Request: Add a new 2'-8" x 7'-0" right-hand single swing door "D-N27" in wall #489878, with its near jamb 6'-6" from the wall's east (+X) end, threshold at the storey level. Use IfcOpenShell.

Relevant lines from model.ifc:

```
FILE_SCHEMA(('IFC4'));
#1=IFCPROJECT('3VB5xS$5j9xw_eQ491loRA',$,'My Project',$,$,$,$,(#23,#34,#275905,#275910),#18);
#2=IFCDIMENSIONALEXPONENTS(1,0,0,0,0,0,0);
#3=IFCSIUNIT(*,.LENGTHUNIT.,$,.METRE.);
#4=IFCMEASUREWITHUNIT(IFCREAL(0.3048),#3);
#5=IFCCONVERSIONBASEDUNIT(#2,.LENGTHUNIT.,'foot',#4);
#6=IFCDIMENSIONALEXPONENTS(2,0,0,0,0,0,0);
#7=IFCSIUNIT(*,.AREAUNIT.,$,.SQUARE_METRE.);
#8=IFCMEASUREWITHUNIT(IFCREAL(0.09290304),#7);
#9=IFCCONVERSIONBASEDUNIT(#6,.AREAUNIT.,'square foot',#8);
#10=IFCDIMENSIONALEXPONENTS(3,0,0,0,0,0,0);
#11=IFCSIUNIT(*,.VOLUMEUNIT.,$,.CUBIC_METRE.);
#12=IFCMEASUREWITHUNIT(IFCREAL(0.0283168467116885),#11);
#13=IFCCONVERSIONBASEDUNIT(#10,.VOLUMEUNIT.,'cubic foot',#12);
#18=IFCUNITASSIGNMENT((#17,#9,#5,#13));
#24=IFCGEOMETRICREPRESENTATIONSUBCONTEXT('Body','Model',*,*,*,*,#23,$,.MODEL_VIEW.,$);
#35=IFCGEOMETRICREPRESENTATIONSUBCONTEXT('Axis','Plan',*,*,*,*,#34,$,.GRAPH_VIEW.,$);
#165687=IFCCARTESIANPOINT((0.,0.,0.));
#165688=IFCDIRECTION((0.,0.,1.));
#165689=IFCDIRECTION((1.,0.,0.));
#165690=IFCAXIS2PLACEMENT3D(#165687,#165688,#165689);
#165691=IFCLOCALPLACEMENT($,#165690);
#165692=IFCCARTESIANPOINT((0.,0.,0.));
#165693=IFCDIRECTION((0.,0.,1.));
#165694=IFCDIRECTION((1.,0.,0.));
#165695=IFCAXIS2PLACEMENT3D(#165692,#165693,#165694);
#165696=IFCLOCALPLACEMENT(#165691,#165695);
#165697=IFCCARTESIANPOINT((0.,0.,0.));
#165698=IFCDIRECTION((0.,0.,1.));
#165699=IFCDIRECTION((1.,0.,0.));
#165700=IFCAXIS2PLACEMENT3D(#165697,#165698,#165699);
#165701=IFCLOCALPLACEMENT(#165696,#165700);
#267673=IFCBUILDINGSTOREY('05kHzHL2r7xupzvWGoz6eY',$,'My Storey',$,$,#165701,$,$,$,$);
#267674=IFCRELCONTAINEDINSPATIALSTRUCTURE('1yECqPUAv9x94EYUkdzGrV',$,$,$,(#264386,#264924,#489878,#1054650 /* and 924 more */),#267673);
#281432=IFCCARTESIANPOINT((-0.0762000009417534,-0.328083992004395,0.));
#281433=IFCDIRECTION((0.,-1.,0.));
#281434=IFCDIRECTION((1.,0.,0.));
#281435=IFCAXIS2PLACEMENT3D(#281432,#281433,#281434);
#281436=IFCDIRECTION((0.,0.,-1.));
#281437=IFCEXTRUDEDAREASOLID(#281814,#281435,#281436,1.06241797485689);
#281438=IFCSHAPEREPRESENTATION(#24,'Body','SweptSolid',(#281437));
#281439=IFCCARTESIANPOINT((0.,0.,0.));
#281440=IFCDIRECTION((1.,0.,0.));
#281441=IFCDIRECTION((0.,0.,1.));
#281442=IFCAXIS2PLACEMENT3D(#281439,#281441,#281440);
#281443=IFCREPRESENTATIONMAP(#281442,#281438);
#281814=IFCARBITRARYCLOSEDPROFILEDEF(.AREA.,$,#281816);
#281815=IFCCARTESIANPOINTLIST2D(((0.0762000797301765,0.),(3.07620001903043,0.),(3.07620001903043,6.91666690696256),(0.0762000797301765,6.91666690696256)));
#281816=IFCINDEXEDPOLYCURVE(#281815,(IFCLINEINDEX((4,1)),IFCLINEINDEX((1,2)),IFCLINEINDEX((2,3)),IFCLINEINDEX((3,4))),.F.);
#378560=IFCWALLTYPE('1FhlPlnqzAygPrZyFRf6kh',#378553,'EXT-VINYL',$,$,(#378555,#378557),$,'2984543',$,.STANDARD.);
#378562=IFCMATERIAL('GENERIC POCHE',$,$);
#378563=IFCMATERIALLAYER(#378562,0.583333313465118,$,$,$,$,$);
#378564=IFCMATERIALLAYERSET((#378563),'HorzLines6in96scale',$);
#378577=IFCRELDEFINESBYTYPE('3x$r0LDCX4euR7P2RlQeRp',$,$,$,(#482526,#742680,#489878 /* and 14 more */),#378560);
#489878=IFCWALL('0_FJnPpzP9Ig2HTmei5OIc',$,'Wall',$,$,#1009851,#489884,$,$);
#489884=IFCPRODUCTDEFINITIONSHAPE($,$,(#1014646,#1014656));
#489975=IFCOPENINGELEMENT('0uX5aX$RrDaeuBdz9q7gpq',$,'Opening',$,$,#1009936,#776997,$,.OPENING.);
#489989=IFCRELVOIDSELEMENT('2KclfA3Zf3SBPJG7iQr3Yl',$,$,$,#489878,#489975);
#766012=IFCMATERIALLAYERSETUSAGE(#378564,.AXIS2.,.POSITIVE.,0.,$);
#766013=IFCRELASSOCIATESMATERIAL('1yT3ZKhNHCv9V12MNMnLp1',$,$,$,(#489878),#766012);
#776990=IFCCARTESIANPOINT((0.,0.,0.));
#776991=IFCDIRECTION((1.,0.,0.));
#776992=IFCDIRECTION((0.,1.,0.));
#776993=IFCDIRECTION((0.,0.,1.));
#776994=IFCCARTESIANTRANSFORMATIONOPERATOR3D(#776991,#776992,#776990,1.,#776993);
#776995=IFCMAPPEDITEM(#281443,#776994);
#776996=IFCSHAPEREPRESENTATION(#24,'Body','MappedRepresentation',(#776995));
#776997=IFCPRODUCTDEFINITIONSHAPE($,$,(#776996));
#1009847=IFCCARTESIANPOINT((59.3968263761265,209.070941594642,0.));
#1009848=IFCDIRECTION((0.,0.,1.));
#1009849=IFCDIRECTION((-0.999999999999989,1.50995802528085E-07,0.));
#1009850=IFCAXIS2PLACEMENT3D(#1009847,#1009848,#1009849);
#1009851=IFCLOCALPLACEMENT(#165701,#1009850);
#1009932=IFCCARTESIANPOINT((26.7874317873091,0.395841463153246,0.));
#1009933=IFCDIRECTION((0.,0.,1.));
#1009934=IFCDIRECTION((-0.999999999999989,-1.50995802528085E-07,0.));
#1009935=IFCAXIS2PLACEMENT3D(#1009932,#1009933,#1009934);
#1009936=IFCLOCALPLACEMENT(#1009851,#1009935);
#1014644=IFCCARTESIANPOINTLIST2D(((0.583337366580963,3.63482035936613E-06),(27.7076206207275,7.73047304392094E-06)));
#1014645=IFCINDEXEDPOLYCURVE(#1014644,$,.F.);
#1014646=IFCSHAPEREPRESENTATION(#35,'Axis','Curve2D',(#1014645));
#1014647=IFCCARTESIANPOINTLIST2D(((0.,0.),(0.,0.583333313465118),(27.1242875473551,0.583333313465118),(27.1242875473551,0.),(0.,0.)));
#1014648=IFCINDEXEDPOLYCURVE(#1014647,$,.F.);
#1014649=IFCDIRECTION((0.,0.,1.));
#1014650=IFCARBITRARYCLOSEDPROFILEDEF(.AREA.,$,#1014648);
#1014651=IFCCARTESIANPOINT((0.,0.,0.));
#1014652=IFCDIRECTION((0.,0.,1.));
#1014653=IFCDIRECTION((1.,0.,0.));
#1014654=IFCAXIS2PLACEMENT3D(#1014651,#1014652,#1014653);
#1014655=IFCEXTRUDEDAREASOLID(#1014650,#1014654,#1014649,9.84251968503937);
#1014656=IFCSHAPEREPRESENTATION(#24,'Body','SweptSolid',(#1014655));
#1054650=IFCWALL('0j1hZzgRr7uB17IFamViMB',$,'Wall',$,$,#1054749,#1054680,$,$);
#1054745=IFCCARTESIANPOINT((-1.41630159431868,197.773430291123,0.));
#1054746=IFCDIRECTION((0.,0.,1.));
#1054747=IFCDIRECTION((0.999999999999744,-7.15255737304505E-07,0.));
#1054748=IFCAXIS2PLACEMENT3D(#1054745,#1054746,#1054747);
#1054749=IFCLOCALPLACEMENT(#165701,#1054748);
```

```python
import numpy as np
import ifcopenshell
import ifcopenshell.api.feature
import ifcopenshell.api.geometry
import ifcopenshell.api.root
import ifcopenshell.api.spatial
import ifcopenshell.geom
import ifcopenshell.util.element
import ifcopenshell.util.placement
import ifcopenshell.util.representation
import ifcopenshell.util.shape
import ifcopenshell.util.unit

model = ifcopenshell.open("model.ifc")
unit_scale = ifcopenshell.util.unit.calculate_unit_scale(model)
settings = ifcopenshell.geom.settings()


def volume(element):
    """Net volume in cubic metres, openings subtracted."""
    shape = ifcopenshell.geom.create_shape(settings, element)
    return ifcopenshell.util.shape.get_volume(shape.geometry)


wall = model.by_guid("0_FJnPpzP9Ig2HTmei5OIc")
storey = ifcopenshell.util.element.get_container(wall, ifc_class="IfcBuildingStorey")
context = ifcopenshell.util.representation.get_context(model, "Model", "Body", "MODEL_VIEW")
before = volume(wall)

width, height, from_end, sill = 0.8128, 2.1336, 1.9812, 0.0  # metres

# The wall runs along its own X axis, and the end named is its -X end.
wall_shape = ifcopenshell.geom.create_shape(settings, wall)
x, y, z = ifcopenshell.util.shape.get_vertices(wall_shape.geometry).T
start = x.min() + from_end
face, thickness = float(y.min()), float(y.max() - y.min())
wall_matrix = ifcopenshell.util.placement.get_local_placement(wall.ObjectPlacement)
level = ifcopenshell.util.placement.get_local_placement(storey.ObjectPlacement)[2, 3]


def in_wall(x, y):
    """Placement at x, y metres in the wall's axes, at sill height."""
    matrix = wall_matrix.copy()
    matrix[:, 3] = wall_matrix @ np.array([x / unit_scale, y / unit_scale, 0.0, 1.0])
    matrix[2, 3] = level + sill / unit_scale
    return matrix


# Opening: a box that overshoots both wall faces by 50 mm.
opening = ifcopenshell.api.root.create_entity(model, ifc_class="IfcOpeningElement", predefined_type="OPENING")
box = ifcopenshell.api.geometry.add_wall_representation(
    model, context=context, length=width, height=height, thickness=thickness + 0.1
)
ifcopenshell.api.geometry.assign_representation(model, product=opening, representation=box)
ifcopenshell.api.geometry.edit_object_placement(model, product=opening, matrix=in_wall(start, face - 0.05), is_si=False)
ifcopenshell.api.feature.add_feature(model, feature=opening, element=wall)

door = ifcopenshell.api.root.create_entity(model, ifc_class="IfcDoor", name="D-N27", predefined_type="DOOR")
door.OverallWidth, door.OverallHeight = width / unit_scale, height / unit_scale
door.OperationType = "SINGLE_SWING_RIGHT"
body = ifcopenshell.api.geometry.add_door_representation(
    model,
    context=context,
    overall_width=door.OverallWidth,
    overall_height=door.OverallHeight,
    operation_type="SINGLE_SWING_RIGHT",
    lining_properties={"LiningDepth": thickness / unit_scale, "ThresholdDepth": thickness / unit_scale},
)
ifcopenshell.api.geometry.assign_representation(model, product=door, representation=body)
ifcopenshell.api.spatial.assign_container(model, products=[door], relating_structure=storey)
ifcopenshell.api.feature.add_filling(model, opening=opening, element=door)

# The lining spans the wall, so the door starts at the wall face.
ifcopenshell.api.geometry.edit_object_placement(model, product=door, matrix=in_wall(start, face), is_si=False)

after = volume(wall)

print(f"wall volume {before:.3f} -> {after:.3f} m3")

model.write("model_edited.ifc")
```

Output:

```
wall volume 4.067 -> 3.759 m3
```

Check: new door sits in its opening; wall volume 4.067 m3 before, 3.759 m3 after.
